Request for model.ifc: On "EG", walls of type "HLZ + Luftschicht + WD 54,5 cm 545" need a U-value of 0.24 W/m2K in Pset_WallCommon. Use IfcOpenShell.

First a look at what the model holds.

```python
import ifcopenshell
import ifcopenshell.util.element

model = ifcopenshell.open("model.ifc")
print(model.schema)
storey = next(s for s in model.by_type("IfcBuildingStorey") if s.Name == "EG")
walls = [e for e in ifcopenshell.util.element.get_decomposition(storey) if e.is_a("IfcWall")]
seen = {}
for e in walls:
    element_type = ifcopenshell.util.element.get_type(e)
    key = (element_type.Name if element_type != e and element_type else None, ifcopenshell.util.element.get_pset(e, "Pset_WallCommon", "ThermalTransmittance"))
    seen[key] = seen.get(key, 0) + 1
for (name, value), count in sorted(seen.items(), key=str):
    print(count, "x", name, "|", value)
```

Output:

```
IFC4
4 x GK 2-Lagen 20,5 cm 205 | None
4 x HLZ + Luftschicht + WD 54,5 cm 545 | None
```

```python
import ifcopenshell
import ifcopenshell.api.pset
import ifcopenshell.util.element

model = ifcopenshell.open("model.ifc")

storey = next(s for s in model.by_type("IfcBuildingStorey") if s.Name == "EG")
walls = [e for e in ifcopenshell.util.element.get_decomposition(storey) if e.is_a("IfcWall")]

count = 0
for e in walls:
    element_type = ifcopenshell.util.element.get_type(e)
    if element_type in (None, e) or element_type.Name != "HLZ + Luftschicht + WD 54,5 cm 545":
        continue
    # add_pset returns the element's existing set when there is one.
    pset = ifcopenshell.api.pset.add_pset(model, product=e, name="Pset_WallCommon")
    ifcopenshell.api.pset.edit_pset(model, pset=pset, properties={"ThermalTransmittance": 0.24})
    count += 1

print(count, "walls updated")

model.write("model_rev.ifc")
```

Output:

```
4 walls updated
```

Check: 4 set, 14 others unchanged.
